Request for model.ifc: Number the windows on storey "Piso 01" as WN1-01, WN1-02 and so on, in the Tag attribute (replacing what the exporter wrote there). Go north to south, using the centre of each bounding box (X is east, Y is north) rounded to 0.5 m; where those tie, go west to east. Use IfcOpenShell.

First a look at what the model holds.

```python
import ifcopenshell
import ifcopenshell.util.element
import ifcopenshell.util.placement

model = ifcopenshell.open("model.ifc")
print(model.schema)
storey = next(s for s in model.by_type("IfcBuildingStorey") if s.Name == "Piso 01")
windows = [e for e in ifcopenshell.util.element.get_decomposition(storey) if e.is_a("IfcWindow")]
for e in sorted(windows, key=lambda e: e.id()):
    origin = ifcopenshell.util.placement.get_local_placement(e.ObjectPlacement)[:3, 3]
    print(e.id(), e.Tag, e.Name, origin.round(2) + 0.0, sep=" | ")
```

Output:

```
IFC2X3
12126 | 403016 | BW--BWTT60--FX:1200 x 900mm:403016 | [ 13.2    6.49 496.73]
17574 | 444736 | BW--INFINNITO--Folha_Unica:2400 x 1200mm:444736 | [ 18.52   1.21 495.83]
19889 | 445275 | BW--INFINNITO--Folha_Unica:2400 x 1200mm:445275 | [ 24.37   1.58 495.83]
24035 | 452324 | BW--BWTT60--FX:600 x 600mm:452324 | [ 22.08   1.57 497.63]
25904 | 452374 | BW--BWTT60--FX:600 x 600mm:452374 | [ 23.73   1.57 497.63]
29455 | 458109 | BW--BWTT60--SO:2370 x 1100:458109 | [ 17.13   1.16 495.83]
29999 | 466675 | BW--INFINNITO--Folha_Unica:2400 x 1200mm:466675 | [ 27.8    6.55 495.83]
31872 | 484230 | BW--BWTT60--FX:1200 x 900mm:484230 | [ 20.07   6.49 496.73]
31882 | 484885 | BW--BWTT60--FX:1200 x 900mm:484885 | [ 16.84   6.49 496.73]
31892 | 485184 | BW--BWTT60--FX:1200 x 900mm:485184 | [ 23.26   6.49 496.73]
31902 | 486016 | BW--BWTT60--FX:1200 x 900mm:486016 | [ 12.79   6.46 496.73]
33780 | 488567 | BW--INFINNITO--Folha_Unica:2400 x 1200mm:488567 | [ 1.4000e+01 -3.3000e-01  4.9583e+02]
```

```python
import ifcopenshell
import ifcopenshell.geom
import ifcopenshell.util.element
import ifcopenshell.util.shape

model = ifcopenshell.open("model.ifc")
settings = ifcopenshell.geom.settings()
settings.set("use-world-coords", True)


def centre(element):
    shape = ifcopenshell.geom.create_shape(settings, element)
    return ifcopenshell.util.shape.get_bbox_centroid(shape.geometry)


storey = next(s for s in model.by_type("IfcBuildingStorey") if s.Name == "Piso 01")
windows = [e for e in ifcopenshell.util.element.get_decomposition(storey) if e.is_a("IfcWindow")]

# Insertion points can sit at a corner or the storey origin, so sort by the geometry (in metres).
centres = {e: centre(e) for e in windows}
windows.sort(key=lambda e: (-round(centres[e][1] / 0.5), centres[e][0]))

for i, e in enumerate(windows, start=1):
    number = f"WN1-{i:02d}"
    e.Tag = number
    print(e.id(), number)

model.write("model-out.ifc")
```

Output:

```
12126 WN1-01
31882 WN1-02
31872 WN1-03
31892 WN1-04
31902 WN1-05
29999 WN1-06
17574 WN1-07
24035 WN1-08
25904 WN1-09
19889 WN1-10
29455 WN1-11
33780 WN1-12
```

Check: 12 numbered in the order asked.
